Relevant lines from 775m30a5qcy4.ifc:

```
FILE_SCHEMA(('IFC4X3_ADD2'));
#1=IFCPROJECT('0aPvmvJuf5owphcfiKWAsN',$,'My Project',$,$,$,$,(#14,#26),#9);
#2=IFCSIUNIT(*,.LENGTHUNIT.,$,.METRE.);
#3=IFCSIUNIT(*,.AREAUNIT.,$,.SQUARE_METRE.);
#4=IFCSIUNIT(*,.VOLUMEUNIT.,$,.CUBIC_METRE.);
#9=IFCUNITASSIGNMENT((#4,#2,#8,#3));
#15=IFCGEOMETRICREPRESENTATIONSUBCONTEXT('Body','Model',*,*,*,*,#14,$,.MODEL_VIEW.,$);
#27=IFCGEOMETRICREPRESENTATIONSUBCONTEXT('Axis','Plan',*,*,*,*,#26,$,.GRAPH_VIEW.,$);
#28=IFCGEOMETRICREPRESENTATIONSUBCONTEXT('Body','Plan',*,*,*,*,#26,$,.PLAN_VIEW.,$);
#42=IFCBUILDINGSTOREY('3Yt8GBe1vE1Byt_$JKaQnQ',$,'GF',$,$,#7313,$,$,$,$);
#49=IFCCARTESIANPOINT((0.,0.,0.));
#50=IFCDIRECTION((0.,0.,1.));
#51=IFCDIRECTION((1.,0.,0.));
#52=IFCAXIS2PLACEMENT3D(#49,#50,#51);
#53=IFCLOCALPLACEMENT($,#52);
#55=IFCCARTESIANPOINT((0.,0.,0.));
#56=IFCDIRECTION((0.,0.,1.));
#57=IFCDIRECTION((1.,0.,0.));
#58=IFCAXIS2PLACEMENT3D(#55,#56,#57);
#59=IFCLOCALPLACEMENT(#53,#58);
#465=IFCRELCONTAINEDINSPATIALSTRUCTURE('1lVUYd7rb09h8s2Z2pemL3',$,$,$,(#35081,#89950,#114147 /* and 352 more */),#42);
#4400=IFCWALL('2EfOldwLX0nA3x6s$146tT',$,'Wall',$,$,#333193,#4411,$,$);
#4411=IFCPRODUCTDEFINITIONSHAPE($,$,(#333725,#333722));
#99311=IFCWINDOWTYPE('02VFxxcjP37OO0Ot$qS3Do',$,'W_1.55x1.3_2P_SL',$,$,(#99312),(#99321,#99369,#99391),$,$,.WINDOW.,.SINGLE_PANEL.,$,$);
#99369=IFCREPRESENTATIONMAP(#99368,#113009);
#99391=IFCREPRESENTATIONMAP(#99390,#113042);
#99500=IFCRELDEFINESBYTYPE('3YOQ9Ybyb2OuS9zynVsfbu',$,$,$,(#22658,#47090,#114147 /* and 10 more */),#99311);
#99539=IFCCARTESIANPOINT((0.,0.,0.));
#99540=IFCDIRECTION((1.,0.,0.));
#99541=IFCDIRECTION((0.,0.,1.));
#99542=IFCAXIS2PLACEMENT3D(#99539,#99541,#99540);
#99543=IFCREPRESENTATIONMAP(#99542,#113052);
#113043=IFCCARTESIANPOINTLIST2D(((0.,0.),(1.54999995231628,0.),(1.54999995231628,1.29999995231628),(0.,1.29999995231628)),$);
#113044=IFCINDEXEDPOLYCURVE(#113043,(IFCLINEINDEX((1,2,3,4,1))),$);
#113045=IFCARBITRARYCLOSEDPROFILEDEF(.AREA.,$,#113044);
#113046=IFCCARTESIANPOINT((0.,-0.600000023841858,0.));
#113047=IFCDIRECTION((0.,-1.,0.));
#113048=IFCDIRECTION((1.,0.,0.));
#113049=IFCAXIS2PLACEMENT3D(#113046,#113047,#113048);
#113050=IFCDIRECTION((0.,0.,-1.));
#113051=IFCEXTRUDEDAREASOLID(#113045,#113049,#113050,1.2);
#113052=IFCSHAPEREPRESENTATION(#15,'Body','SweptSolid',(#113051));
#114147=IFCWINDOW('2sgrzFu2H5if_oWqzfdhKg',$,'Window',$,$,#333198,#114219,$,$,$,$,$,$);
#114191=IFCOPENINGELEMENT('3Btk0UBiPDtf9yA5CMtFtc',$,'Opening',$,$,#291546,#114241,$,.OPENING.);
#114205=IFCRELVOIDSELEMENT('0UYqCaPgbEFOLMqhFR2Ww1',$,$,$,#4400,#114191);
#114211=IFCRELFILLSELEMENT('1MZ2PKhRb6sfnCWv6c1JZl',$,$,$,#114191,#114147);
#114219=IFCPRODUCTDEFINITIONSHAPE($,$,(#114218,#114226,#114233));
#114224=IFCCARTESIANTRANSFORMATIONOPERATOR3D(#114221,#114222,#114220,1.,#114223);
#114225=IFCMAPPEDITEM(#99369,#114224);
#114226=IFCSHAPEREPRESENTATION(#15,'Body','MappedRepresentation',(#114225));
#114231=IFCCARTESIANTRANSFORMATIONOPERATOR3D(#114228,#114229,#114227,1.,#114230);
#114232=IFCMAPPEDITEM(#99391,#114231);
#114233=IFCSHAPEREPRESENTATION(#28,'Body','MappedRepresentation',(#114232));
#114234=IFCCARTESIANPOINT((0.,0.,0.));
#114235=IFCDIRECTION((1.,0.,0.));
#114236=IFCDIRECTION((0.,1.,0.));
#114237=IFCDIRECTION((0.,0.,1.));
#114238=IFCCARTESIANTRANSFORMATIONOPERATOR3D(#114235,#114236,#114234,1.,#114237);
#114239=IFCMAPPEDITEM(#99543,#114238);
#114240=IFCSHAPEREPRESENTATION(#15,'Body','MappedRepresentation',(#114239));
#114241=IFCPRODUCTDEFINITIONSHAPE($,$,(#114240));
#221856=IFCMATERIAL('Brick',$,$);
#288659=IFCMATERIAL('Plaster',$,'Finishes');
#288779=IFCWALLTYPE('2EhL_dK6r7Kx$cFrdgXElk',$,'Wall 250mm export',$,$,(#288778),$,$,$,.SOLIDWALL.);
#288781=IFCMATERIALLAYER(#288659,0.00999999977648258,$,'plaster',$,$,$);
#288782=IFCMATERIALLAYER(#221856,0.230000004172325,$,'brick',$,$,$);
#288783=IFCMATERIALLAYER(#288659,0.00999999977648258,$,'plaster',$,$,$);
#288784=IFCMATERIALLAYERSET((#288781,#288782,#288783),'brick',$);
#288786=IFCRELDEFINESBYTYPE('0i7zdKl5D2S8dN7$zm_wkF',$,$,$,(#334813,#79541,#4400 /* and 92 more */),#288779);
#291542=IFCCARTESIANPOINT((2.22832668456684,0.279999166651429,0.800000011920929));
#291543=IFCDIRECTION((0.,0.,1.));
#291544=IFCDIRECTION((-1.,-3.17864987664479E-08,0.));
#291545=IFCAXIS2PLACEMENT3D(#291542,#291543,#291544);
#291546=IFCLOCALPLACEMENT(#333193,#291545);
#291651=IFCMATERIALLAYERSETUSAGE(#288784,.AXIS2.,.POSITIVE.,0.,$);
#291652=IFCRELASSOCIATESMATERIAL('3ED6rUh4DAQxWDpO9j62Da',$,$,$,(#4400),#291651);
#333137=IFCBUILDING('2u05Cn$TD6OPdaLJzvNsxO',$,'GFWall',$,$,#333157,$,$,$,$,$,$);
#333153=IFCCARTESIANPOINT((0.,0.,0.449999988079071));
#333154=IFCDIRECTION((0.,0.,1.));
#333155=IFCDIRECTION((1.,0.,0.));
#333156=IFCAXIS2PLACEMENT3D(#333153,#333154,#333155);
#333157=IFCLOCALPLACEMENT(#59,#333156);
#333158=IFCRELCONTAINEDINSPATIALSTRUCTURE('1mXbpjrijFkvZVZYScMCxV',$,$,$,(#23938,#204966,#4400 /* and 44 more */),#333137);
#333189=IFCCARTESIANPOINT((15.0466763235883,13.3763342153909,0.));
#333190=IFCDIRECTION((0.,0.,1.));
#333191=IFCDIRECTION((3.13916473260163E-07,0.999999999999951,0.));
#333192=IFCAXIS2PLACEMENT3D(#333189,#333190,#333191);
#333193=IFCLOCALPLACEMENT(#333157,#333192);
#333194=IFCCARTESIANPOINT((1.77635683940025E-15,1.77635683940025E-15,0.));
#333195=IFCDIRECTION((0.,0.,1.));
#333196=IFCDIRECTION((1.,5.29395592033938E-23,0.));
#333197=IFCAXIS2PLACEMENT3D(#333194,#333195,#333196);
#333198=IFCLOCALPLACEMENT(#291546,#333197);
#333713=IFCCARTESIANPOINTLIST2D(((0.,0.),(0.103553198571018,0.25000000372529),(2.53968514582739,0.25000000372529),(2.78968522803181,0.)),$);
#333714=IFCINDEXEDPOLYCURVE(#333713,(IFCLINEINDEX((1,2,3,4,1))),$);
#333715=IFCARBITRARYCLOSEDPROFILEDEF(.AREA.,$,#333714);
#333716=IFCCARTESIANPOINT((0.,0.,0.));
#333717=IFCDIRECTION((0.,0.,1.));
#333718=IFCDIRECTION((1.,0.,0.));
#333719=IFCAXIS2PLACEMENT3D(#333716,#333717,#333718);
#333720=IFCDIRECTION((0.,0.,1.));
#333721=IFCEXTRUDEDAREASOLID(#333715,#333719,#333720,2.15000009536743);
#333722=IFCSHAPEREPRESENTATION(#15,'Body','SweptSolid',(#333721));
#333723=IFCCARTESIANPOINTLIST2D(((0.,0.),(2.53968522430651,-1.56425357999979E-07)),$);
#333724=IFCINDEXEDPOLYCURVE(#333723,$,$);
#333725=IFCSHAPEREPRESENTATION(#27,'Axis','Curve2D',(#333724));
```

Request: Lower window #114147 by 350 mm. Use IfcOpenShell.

```python
import numpy as np
import ifcopenshell
import ifcopenshell.api.geometry
import ifcopenshell.util.placement
import ifcopenshell.util.unit

model = ifcopenshell.open("775m30a5qcy4.ifc")
unit_scale = ifcopenshell.util.unit.calculate_unit_scale(model)

window = model.by_guid("2sgrzFu2H5if_oWqzfdhKg")
opening = window.FillsVoids[0].RelatingOpeningElement
dz = -0.35

shift = np.array([0.0, 0.0, dz])
# The window is placed relative to its opening, so it follows when the opening moves.
matrix = ifcopenshell.util.placement.get_local_placement(opening.ObjectPlacement)
matrix[:3, 3] += shift
ifcopenshell.api.geometry.edit_object_placement(
    model, product=opening, matrix=matrix, is_si=False, should_transform_children=True
)

print(f"moved by {dz * unit_scale:+.3f} m")

model.write("775m30a5qcy4_edited.ifc")
```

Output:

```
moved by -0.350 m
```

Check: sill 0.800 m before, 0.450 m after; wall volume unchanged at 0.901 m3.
